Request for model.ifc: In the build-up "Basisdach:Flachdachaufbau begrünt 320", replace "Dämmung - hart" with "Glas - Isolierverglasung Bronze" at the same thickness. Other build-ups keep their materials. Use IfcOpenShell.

First a look at what the model holds.

```python
import ifcopenshell
import ifcopenshell.util.element

model = ifcopenshell.open("model.ifc")
print(model.schema)
for layer_set in model.by_type("IfcMaterialLayerSet"):
    if layer_set.LayerSetName == "Basisdach:Flachdachaufbau begrünt 320":
        for layer in layer_set.MaterialLayers:
            print(layer.id(), layer.Material and layer.Material.Name, layer.LayerThickness, sep=" | ")
        print(len(ifcopenshell.util.element.get_elements_by_material(model, layer_set)), "elements and types use it")
print(sorted(m.Name for m in model.by_type("IfcMaterial") if m.Name)[:60])
```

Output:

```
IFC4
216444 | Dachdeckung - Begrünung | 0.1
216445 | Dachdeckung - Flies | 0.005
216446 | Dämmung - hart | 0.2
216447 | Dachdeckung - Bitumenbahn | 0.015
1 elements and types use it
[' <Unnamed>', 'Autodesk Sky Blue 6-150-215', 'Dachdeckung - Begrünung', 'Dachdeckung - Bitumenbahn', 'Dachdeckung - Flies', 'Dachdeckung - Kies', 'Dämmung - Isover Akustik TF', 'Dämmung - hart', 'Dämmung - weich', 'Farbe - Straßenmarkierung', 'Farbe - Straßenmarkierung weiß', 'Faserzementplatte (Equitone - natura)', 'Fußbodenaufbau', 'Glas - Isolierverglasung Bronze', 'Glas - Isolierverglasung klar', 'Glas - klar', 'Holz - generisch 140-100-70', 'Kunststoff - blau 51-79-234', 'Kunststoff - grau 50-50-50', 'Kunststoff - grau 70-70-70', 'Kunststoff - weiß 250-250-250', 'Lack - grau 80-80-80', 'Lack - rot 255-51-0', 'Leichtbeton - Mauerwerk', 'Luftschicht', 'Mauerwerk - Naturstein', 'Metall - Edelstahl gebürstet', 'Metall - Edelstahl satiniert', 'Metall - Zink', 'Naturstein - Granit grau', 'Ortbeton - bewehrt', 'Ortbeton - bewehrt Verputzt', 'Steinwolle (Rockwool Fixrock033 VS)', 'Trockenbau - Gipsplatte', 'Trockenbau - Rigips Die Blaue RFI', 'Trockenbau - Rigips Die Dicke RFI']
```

```python
import ifcopenshell
import ifcopenshell.api.material

model = ifcopenshell.open("model.ifc")

layer_set = next(s for s in model.by_type("IfcMaterialLayerSet") if s.LayerSetName == "Basisdach:Flachdachaufbau begrünt 320")
layer = next(l for l in layer_set.MaterialLayers if l.Material and l.Material.Name == "Dämmung - hart")
material = next(m for m in model.by_type("IfcMaterial") if m.Name == "Glas - Isolierverglasung Bronze")

# Point this one layer at the other material; renaming the old one would change it everywhere.
ifcopenshell.api.material.edit_layer(model, layer=layer, attributes={"Name": material.Name}, material=material)

print([l.Material.Name if l.Material else None for l in layer_set.MaterialLayers])

model.write("model_rev.ifc")
```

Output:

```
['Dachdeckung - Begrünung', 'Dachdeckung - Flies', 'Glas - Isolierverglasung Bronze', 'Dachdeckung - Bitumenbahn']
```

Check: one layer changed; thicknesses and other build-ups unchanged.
